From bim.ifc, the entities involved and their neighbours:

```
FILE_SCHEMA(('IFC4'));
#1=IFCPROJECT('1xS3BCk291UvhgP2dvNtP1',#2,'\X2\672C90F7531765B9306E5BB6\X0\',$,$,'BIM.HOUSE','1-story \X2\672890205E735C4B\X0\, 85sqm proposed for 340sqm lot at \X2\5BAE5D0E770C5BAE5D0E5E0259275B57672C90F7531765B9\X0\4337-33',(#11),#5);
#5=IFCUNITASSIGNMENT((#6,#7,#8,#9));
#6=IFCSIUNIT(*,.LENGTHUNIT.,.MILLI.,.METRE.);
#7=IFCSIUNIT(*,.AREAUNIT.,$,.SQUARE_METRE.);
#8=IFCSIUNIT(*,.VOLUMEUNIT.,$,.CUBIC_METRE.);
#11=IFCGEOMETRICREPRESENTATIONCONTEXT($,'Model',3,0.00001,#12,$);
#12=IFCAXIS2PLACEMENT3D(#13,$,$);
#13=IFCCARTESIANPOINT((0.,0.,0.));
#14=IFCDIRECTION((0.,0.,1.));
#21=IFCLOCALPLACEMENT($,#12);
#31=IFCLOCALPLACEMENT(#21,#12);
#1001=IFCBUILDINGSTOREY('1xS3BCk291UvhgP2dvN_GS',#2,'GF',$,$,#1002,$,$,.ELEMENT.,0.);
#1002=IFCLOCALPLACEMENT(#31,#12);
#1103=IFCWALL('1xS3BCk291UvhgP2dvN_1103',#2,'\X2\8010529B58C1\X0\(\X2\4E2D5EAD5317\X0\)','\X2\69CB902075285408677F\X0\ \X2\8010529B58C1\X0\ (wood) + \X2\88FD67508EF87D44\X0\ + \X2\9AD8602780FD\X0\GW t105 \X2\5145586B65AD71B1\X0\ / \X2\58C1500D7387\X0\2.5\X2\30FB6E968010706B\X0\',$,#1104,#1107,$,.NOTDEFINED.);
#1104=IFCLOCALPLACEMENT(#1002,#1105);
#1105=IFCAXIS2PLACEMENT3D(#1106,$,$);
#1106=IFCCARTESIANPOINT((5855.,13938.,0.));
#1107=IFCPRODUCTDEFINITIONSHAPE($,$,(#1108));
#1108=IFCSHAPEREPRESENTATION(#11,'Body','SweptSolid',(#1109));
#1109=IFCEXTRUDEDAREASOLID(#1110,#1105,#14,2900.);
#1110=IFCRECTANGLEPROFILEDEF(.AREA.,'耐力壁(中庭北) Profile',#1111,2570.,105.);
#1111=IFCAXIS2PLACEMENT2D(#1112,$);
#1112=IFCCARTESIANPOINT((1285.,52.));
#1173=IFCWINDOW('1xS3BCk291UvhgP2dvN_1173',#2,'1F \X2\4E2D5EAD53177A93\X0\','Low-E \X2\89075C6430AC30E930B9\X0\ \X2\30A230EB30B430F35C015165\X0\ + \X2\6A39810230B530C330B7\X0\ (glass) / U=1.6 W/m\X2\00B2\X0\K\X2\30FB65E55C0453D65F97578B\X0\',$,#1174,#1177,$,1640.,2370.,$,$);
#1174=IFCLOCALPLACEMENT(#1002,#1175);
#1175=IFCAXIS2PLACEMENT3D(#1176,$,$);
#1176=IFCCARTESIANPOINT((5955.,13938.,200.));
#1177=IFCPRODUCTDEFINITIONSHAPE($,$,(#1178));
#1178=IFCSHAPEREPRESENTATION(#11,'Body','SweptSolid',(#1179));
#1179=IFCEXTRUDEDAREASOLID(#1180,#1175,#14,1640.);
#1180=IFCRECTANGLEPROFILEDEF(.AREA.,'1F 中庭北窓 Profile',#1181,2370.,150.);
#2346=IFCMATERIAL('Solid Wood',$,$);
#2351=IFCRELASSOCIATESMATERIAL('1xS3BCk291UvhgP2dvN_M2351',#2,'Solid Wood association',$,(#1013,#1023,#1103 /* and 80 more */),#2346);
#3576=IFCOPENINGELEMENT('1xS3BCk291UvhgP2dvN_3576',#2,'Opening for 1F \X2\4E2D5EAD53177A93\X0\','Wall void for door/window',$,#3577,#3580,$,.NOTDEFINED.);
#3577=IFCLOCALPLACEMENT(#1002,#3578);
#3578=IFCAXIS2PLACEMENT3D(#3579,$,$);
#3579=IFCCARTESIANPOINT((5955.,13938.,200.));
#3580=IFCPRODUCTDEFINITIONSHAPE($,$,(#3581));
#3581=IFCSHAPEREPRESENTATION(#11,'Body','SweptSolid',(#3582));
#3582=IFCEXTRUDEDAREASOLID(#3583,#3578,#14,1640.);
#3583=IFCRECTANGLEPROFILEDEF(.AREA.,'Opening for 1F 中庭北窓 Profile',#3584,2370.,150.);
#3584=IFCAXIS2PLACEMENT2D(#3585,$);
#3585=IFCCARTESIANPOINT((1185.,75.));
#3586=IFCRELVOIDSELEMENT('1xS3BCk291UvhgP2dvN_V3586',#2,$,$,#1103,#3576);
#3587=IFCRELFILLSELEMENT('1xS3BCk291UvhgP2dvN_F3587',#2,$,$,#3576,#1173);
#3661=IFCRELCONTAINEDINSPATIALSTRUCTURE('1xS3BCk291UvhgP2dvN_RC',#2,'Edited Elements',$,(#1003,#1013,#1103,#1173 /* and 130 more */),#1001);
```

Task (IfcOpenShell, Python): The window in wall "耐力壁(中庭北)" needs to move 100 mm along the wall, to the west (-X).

```python
import ifcopenshell
import ifcopenshell.api.geometry
import ifcopenshell.util.placement

model = ifcopenshell.open("bim.ifc")

window = model.by_guid("1xS3BCk291UvhgP2dvN_1173")
opening = window.FillsVoids[0].RelatingOpeningElement
wall = opening.VoidsElements[0].RelatingBuildingElement

wall_matrix = ifcopenshell.util.placement.get_local_placement(wall.ObjectPlacement)
shift = wall_matrix[:3, 0] * -100.0
before = ifcopenshell.util.placement.get_local_placement(window.ObjectPlacement)[:3, 3].copy()

# The window is not placed relative to its opening, so move both.
for product in (opening, window):
    matrix = ifcopenshell.util.placement.get_local_placement(product.ObjectPlacement)
    matrix[:3, 3] += shift
    ifcopenshell.api.geometry.edit_object_placement(model, product=product, matrix=matrix, is_si=False)

after = ifcopenshell.util.placement.get_local_placement(window.ObjectPlacement)[:3, 3]
print("window moved by", (after - before).round(3) + 0.0)

model.write("bim_updated.ifc")
```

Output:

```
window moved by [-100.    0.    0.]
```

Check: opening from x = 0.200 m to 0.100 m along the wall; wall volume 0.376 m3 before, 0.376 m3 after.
